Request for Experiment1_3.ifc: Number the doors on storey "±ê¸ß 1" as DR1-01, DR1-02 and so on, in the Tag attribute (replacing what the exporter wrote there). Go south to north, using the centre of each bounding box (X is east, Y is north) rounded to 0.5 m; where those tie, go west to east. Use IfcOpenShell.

First a look at what the model holds.

```python
import ifcopenshell
import ifcopenshell.util.element
import ifcopenshell.util.placement

model = ifcopenshell.open("Experiment1_3.ifc")
print(model.schema)
storey = next(s for s in model.by_type("IfcBuildingStorey") if s.Name == "±ê¸ß 1")
doors = [e for e in ifcopenshell.util.element.get_decomposition(storey) if e.is_a("IfcDoor")]
for e in sorted(doors, key=lambda e: e.id()):
    origin = ifcopenshell.util.placement.get_local_placement(e.ObjectPlacement)[:3, 3]
    print(e.id(), e.Tag, e.Name, origin.round(2) + 0.0, sep=" | ")
```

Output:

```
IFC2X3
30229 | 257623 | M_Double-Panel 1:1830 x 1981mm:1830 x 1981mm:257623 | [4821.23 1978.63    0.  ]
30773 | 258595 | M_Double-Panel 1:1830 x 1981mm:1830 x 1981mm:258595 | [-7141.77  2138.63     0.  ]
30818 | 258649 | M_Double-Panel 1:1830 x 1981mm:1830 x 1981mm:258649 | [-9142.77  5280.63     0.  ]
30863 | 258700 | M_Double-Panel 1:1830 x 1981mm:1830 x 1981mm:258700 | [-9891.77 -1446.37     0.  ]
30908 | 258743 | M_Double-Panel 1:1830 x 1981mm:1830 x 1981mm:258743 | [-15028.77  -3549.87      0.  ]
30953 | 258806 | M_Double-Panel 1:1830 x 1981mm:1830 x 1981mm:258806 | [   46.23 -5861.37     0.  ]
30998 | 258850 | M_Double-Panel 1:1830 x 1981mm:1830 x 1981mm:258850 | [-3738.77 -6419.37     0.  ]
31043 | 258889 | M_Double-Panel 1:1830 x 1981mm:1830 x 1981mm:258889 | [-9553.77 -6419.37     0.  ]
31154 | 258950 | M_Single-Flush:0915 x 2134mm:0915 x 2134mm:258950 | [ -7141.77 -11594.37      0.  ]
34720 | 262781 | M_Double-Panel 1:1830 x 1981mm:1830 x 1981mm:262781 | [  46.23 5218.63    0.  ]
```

```python
import ifcopenshell
import ifcopenshell.geom
import ifcopenshell.util.element
import ifcopenshell.util.shape

model = ifcopenshell.open("Experiment1_3.ifc")
settings = ifcopenshell.geom.settings()
settings.set("use-world-coords", True)


def centre(element):
    shape = ifcopenshell.geom.create_shape(settings, element)
    return ifcopenshell.util.shape.get_bbox_centroid(shape.geometry)


storey = next(s for s in model.by_type("IfcBuildingStorey") if s.Name == "±ê¸ß 1")
doors = [e for e in ifcopenshell.util.element.get_decomposition(storey) if e.is_a("IfcDoor")]

# Insertion points can sit at a corner or the storey origin, so sort by the geometry (in metres).
centres = {e: centre(e) for e in doors}
doors.sort(key=lambda e: (round(centres[e][1] / 0.5), centres[e][0]))

for i, e in enumerate(doors, start=1):
    number = f"DR1-{i:02d}"
    e.Tag = number
    print(e.id(), number)

model.write("Experiment1_3_updated.ifc")
```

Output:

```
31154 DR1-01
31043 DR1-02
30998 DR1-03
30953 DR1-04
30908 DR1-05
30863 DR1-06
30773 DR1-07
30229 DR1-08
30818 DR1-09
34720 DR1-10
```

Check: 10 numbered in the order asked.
